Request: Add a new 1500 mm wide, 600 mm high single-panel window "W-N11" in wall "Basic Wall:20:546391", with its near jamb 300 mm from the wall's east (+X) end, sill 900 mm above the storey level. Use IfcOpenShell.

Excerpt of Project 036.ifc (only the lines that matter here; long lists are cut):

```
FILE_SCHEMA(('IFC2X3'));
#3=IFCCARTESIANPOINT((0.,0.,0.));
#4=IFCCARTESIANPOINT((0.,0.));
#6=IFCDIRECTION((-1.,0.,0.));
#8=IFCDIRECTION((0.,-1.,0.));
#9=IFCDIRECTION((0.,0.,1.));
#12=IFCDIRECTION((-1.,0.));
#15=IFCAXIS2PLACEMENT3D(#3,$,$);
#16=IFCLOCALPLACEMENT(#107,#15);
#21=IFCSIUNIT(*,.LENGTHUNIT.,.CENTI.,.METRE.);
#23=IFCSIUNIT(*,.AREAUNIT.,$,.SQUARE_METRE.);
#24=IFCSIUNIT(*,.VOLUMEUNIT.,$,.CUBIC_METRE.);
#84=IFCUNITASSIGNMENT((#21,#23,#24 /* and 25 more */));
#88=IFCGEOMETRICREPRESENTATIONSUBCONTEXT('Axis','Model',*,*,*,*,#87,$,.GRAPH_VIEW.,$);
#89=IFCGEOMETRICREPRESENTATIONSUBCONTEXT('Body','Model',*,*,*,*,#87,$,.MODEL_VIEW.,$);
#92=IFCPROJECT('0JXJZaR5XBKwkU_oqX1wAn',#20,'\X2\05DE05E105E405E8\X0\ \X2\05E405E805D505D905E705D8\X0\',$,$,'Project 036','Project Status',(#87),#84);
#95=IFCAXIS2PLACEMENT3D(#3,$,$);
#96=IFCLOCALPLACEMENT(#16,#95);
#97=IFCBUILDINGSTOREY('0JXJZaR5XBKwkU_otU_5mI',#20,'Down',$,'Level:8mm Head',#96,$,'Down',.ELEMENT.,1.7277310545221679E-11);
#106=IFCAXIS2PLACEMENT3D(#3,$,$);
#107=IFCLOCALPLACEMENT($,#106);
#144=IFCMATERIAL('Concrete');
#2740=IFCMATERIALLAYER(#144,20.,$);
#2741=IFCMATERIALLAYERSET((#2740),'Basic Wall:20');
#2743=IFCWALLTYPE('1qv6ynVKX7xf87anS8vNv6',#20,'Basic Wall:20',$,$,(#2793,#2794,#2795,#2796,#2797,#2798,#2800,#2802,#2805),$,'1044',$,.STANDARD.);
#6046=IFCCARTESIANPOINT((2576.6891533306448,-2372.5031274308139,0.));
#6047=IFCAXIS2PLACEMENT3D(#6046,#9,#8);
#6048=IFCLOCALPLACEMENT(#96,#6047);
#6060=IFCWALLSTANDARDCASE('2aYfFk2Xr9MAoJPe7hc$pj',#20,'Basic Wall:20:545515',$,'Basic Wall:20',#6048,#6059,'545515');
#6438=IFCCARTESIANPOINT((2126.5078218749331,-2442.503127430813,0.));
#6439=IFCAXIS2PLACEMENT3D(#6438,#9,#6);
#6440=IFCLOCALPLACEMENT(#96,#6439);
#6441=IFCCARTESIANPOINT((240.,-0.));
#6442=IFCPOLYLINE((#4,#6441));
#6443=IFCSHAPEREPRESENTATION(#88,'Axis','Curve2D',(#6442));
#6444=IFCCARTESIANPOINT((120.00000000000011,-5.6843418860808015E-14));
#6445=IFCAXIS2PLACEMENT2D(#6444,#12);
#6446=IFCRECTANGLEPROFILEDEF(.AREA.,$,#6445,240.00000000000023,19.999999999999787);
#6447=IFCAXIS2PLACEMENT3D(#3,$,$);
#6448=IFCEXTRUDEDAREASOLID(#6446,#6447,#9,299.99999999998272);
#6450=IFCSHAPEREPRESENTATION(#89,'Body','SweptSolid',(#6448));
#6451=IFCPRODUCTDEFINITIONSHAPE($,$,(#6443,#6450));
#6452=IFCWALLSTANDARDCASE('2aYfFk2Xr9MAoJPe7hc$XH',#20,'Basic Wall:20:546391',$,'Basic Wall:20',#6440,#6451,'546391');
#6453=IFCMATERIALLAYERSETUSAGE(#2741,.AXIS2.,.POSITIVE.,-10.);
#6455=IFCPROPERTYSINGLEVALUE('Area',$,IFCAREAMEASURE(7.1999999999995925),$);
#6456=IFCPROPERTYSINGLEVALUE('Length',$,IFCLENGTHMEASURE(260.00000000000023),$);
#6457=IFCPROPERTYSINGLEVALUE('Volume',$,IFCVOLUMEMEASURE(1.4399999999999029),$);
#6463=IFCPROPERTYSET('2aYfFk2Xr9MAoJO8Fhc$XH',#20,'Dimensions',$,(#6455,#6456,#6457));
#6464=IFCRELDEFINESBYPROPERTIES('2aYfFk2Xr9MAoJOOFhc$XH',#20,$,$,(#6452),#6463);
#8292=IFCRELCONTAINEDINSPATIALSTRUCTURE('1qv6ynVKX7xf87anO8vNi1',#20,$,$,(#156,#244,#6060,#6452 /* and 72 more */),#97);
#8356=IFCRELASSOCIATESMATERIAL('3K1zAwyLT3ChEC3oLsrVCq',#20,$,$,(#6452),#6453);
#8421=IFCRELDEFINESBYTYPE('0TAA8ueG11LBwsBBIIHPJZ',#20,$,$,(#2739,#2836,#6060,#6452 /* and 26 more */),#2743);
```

```python
import numpy as np
import ifcopenshell
import ifcopenshell.api.feature
import ifcopenshell.api.geometry
import ifcopenshell.api.pset
import ifcopenshell.api.root
import ifcopenshell.api.spatial
import ifcopenshell.api.type
import ifcopenshell.geom
import ifcopenshell.util.element
import ifcopenshell.util.placement
import ifcopenshell.util.representation
import ifcopenshell.util.shape
import ifcopenshell.util.unit

model = ifcopenshell.open("Project 036.ifc")
unit_scale = ifcopenshell.util.unit.calculate_unit_scale(model)
area_scale = ifcopenshell.util.unit.calculate_unit_scale(model, "AREAUNIT")
volume_scale = ifcopenshell.util.unit.calculate_unit_scale(model, "VOLUMEUNIT")
settings = ifcopenshell.geom.settings()


def volume(element):
    """Net volume in cubic metres, openings subtracted."""
    shape = ifcopenshell.geom.create_shape(settings, element)
    return ifcopenshell.util.shape.get_volume(shape.geometry)


wall = model.by_guid("2aYfFk2Xr9MAoJPe7hc$XH")
storey = ifcopenshell.util.element.get_container(wall, ifc_class="IfcBuildingStorey")
context = ifcopenshell.util.representation.get_context(model, "Model", "Body", "MODEL_VIEW")
before = volume(wall)

width, height, from_end, sill = 1.5, 0.6, 0.3, 0.9  # metres

# The wall runs along its own X axis, and the end named is its -X end.
wall_shape = ifcopenshell.geom.create_shape(settings, wall)
x, y, z = ifcopenshell.util.shape.get_vertices(wall_shape.geometry).T
start = x.min() + from_end
face, thickness = float(y.min()), float(y.max() - y.min())
wall_matrix = ifcopenshell.util.placement.get_local_placement(wall.ObjectPlacement)
level = ifcopenshell.util.placement.get_local_placement(storey.ObjectPlacement)[2, 3]


def in_wall(x, y):
    """Placement at x, y metres in the wall's axes, at sill height."""
    matrix = wall_matrix.copy()
    matrix[:, 3] = wall_matrix @ np.array([x / unit_scale, y / unit_scale, 0.0, 1.0])
    matrix[2, 3] = level + sill / unit_scale
    return matrix


# Opening: a box that overshoots both wall faces by 50 mm.
opening = ifcopenshell.api.root.create_entity(model, ifc_class="IfcOpeningElement")
box = ifcopenshell.api.geometry.add_wall_representation(
    model, context=context, length=width, height=height, thickness=thickness + 0.1
)
ifcopenshell.api.geometry.assign_representation(model, product=opening, representation=box)
ifcopenshell.api.geometry.edit_object_placement(model, product=opening, matrix=in_wall(start, face - 0.05), is_si=False)
ifcopenshell.api.feature.add_feature(model, feature=opening, element=wall)

window = ifcopenshell.api.root.create_entity(model, ifc_class="IfcWindow", name="W-N11")
window.OverallWidth, window.OverallHeight = width / unit_scale, height / unit_scale
body = ifcopenshell.api.geometry.add_window_representation(
    model,
    context=context,
    overall_width=window.OverallWidth,
    overall_height=window.OverallHeight,
    partition_type="SINGLE_PANEL",
)
ifcopenshell.api.geometry.assign_representation(model, product=window, representation=body)
ifcopenshell.api.spatial.assign_container(model, products=[window], relating_structure=storey)
fills = ifcopenshell.api.feature.add_filling(model, opening=opening, element=window)
fills.OwnerHistory = window.OwnerHistory  # required in IFC2X3

# IFC2X3 keeps the operation on the window style.
style = ifcopenshell.api.root.create_entity(model, ifc_class="IfcWindowStyle", name="W-N11")
style.OperationType, style.ConstructionType = "SINGLE_PANEL", "NOTDEFINED"
style.ParameterTakesPrecedence = style.Sizeable = False
ifcopenshell.api.type.assign_type(model, related_objects=[window], relating_type=style)

# Centre the window in the wall's thickness.
ifcopenshell.api.geometry.edit_object_placement(model, product=window, matrix=in_wall(start, face), is_si=False)
window_shape = ifcopenshell.geom.create_shape(settings, window)
depth = ifcopenshell.util.shape.get_vertices(window_shape.geometry)[:, 1]
offset = face + thickness / 2 - (depth.min() + depth.max()) / 2
ifcopenshell.api.geometry.edit_object_placement(model, product=window, matrix=in_wall(start, offset), is_si=False)

after = volume(wall)

# Update the wall's stored quantities.
pset = model.by_id(ifcopenshell.util.element.get_pset(wall, "Dimensions", should_inherit=False)["id"])
ifcopenshell.api.pset.edit_pset(model, pset=pset, properties={
    "Area": model.create_entity("IfcAreaMeasure", after / thickness / area_scale),
    "Volume": model.create_entity("IfcVolumeMeasure", after / volume_scale),
})

print(f"wall volume {before:.3f} -> {after:.3f} m3")

model.write("Project 036_rev.ifc")
```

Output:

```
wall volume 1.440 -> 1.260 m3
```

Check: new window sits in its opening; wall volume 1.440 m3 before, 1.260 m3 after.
